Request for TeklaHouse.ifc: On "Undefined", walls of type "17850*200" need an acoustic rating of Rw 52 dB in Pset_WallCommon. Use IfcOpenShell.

First a look at what the model holds.

```python
import ifcopenshell
import ifcopenshell.util.element

model = ifcopenshell.open("TeklaHouse.ifc")
print(model.schema)
storey = next(s for s in model.by_type("IfcBuildingStorey") if s.Name == "Undefined")
walls = [e for e in ifcopenshell.util.element.get_decomposition(storey) if e.is_a("IfcWall")]
seen = {}
for e in walls:
    element_type = ifcopenshell.util.element.get_type(e)
    key = (element_type.Name if element_type != e and element_type else None, ifcopenshell.util.element.get_pset(e, "Pset_WallCommon", "AcousticRating"))
    seen[key] = seen.get(key, 0) + 1
for (name, value), count in sorted(seen.items(), key=str):
    print(count, "x", name, "|", value)
```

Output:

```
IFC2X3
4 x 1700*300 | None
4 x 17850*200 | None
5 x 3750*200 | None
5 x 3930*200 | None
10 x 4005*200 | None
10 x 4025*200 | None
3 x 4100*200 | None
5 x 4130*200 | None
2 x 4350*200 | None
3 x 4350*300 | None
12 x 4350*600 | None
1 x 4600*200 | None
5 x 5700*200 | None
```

```python
import ifcopenshell
import ifcopenshell.api.pset
import ifcopenshell.util.element

model = ifcopenshell.open("TeklaHouse.ifc")

storey = next(s for s in model.by_type("IfcBuildingStorey") if s.Name == "Undefined")
walls = [e for e in ifcopenshell.util.element.get_decomposition(storey) if e.is_a("IfcWall")]

count = 0
for e in walls:
    element_type = ifcopenshell.util.element.get_type(e)
    if element_type in (None, e) or element_type.Name != "17850*200":
        continue
    # add_pset returns the element's existing set when there is one.
    pset = ifcopenshell.api.pset.add_pset(model, product=e, name="Pset_WallCommon")
    ifcopenshell.api.pset.edit_pset(model, pset=pset, properties={"AcousticRating": "Rw 52 dB"})
    count += 1

print(count, "walls updated")

model.write("TeklaHouse_edited.ifc")
```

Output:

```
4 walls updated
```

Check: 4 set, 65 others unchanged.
